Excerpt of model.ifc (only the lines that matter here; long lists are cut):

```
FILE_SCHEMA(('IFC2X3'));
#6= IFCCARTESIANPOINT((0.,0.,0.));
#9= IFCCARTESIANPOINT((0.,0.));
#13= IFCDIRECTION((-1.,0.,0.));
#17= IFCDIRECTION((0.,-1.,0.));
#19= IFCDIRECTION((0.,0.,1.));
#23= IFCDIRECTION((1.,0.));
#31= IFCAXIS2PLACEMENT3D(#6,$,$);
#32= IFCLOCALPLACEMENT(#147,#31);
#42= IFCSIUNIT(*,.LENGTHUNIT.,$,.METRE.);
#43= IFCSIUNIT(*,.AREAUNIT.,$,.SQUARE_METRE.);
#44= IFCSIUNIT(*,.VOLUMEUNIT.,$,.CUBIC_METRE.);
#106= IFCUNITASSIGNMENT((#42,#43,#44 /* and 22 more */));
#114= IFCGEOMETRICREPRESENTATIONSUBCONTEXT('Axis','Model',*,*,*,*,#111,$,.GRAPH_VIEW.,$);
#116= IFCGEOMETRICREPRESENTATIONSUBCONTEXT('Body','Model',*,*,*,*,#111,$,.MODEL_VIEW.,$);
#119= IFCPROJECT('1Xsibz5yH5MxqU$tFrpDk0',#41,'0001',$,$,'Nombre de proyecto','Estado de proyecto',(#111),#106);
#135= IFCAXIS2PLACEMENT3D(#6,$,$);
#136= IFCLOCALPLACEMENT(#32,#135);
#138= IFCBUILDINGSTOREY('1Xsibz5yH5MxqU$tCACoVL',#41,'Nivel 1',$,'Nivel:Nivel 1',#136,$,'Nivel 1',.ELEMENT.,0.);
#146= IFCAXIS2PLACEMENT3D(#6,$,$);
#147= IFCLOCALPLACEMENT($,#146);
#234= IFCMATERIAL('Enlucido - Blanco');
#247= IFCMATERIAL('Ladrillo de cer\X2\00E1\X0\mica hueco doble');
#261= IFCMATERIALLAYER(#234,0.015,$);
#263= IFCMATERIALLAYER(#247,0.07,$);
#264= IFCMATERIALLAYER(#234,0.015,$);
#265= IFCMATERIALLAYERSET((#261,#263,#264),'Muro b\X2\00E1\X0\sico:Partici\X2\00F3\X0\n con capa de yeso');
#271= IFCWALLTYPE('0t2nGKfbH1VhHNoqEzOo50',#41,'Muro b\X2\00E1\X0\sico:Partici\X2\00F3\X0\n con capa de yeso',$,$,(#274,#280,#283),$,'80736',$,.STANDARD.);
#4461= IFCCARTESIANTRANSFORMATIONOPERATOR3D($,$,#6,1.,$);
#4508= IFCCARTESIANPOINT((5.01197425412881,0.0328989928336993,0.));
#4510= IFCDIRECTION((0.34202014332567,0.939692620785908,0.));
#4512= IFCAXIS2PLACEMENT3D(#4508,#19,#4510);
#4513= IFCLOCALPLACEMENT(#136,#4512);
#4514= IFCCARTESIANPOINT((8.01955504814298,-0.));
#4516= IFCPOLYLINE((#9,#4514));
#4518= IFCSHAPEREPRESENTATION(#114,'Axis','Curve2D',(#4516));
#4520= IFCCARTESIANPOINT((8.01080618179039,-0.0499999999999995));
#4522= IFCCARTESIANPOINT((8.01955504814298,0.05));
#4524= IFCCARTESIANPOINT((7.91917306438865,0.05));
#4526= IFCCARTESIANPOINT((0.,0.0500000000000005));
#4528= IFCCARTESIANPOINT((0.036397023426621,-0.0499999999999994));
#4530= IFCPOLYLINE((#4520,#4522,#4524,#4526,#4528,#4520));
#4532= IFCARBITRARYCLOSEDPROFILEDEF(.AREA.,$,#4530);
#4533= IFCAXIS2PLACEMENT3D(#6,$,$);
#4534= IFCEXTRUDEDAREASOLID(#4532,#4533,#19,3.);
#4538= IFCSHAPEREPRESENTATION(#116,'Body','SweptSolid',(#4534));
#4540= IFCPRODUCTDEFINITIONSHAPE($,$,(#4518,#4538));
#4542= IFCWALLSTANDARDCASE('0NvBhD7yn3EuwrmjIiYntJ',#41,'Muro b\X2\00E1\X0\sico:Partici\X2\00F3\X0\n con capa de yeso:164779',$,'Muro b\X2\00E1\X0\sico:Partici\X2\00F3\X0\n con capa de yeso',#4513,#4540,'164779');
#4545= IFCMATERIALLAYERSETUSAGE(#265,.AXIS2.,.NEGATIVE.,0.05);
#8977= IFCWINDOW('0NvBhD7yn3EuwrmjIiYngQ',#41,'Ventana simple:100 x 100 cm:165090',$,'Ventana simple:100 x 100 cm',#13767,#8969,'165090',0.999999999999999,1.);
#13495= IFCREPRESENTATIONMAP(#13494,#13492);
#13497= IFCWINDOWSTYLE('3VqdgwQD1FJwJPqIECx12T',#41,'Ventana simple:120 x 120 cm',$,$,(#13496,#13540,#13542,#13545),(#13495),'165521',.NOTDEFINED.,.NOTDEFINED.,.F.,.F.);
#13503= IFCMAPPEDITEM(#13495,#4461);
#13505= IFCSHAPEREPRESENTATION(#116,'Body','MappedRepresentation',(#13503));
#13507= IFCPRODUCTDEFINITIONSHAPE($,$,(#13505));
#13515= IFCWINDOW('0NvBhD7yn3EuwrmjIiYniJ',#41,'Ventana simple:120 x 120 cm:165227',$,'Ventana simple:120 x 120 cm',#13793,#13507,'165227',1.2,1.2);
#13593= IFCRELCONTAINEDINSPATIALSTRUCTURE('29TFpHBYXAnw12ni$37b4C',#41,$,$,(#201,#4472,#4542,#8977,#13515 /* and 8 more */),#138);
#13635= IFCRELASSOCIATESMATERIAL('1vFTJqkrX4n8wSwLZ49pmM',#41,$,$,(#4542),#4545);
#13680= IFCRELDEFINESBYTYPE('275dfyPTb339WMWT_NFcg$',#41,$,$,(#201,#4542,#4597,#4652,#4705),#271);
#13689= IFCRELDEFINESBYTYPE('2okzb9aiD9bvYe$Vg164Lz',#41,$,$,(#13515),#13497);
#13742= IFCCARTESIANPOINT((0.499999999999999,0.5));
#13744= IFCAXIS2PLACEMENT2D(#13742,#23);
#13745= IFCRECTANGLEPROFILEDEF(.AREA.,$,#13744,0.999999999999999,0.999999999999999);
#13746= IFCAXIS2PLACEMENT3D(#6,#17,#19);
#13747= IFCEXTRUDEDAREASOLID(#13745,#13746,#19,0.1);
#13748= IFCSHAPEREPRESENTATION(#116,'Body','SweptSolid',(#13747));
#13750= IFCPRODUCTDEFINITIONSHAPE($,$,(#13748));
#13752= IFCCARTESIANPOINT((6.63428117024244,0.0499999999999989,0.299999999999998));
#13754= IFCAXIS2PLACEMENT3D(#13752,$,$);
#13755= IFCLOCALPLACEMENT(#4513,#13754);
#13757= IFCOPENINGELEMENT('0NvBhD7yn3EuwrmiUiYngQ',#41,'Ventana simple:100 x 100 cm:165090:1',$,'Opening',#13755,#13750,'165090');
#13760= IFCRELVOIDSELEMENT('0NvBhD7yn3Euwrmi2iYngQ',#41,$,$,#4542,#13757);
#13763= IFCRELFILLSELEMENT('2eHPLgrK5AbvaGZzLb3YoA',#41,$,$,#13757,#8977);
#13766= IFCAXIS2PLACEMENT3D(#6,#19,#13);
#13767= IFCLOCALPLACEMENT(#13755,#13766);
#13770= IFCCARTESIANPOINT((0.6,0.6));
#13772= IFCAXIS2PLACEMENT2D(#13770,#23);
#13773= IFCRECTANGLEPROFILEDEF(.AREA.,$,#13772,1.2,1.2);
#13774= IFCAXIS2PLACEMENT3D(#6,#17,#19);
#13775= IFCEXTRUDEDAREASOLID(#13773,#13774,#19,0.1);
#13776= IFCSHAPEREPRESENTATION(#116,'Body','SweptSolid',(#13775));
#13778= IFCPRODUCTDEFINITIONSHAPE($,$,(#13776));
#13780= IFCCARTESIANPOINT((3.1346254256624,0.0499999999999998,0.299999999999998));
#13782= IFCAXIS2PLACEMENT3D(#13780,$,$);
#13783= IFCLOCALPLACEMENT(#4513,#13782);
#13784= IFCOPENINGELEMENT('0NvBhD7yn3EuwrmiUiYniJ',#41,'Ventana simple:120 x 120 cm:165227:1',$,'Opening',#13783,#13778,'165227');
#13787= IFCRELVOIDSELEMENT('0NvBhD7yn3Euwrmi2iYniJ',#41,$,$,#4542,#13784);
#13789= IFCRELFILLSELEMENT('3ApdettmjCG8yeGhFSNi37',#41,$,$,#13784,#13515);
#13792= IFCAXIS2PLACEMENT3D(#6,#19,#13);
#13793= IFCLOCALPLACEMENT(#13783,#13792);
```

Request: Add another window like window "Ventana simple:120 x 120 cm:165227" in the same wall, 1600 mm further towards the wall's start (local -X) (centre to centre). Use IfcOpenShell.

```python
import ifcopenshell
import ifcopenshell.api.feature
import ifcopenshell.api.geometry
import ifcopenshell.api.root
import ifcopenshell.geom
import ifcopenshell.util.element
import ifcopenshell.util.placement
import ifcopenshell.util.shape
import ifcopenshell.util.unit

model = ifcopenshell.open("model.ifc")
unit_scale = ifcopenshell.util.unit.calculate_unit_scale(model)
settings = ifcopenshell.geom.settings()


def volume(element):
    """Net volume in cubic metres, openings subtracted."""
    shape = ifcopenshell.geom.create_shape(settings, element)
    return ifcopenshell.util.shape.get_volume(shape.geometry)


def reuse_history(source, copy):
    """copy_class also copies each property set's owner history, people and application; keep the originals."""
    for rel in copy.IsDefinedBy:
        if rel.is_a("IfcRelDefinesByProperties") and (history := rel.RelatingPropertyDefinition.OwnerHistory):
            rel.RelatingPropertyDefinition.OwnerHistory = source.OwnerHistory
            ifcopenshell.util.element.remove_deep2(model, history)


window = model.by_guid("0NvBhD7yn3EuwrmjIiYniJ")
opening = window.FillsVoids[0].RelatingOpeningElement
wall = opening.VoidsElements[0].RelatingBuildingElement
before = volume(wall)
shift = ifcopenshell.util.placement.get_local_placement(wall.ObjectPlacement)[:3, 0] * -1.6 / unit_scale

# copy_class copies the void relationship, type, container and properties, but no geometry.
new_opening = ifcopenshell.api.root.copy_class(model, product=opening)
new_opening.Representation = ifcopenshell.util.element.copy_deep(
    model, opening.Representation, exclude=["IfcGeometricRepresentationContext", "IfcRepresentationMap"]
)
new_opening.Name = "Ventana simple:120 x 120 cm"
new_opening.Tag = None
new_window = ifcopenshell.api.root.copy_class(model, product=window)
new_window.Representation = ifcopenshell.util.element.copy_deep(
    model, window.Representation, exclude=["IfcGeometricRepresentationContext", "IfcRepresentationMap"]
)
new_window.Name = "Ventana simple:120 x 120 cm"
new_window.Tag = None
reuse_history(window, new_window)
fills = ifcopenshell.api.feature.add_filling(model, opening=new_opening, element=new_window)
fills.OwnerHistory = new_window.OwnerHistory  # required in IFC2X3

for old, new in ((opening, new_opening), (window, new_window)):
    matrix = ifcopenshell.util.placement.get_local_placement(old.ObjectPlacement)
    matrix[:3, 3] += shift
    ifcopenshell.api.geometry.edit_object_placement(model, product=new, matrix=matrix, is_si=False)

after = volume(wall)

print(f"wall volume {before:.3f} -> {after:.3f} m3")

model.write("model_rev.ifc")
```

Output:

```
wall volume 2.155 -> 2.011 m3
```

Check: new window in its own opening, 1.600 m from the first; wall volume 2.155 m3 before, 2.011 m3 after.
